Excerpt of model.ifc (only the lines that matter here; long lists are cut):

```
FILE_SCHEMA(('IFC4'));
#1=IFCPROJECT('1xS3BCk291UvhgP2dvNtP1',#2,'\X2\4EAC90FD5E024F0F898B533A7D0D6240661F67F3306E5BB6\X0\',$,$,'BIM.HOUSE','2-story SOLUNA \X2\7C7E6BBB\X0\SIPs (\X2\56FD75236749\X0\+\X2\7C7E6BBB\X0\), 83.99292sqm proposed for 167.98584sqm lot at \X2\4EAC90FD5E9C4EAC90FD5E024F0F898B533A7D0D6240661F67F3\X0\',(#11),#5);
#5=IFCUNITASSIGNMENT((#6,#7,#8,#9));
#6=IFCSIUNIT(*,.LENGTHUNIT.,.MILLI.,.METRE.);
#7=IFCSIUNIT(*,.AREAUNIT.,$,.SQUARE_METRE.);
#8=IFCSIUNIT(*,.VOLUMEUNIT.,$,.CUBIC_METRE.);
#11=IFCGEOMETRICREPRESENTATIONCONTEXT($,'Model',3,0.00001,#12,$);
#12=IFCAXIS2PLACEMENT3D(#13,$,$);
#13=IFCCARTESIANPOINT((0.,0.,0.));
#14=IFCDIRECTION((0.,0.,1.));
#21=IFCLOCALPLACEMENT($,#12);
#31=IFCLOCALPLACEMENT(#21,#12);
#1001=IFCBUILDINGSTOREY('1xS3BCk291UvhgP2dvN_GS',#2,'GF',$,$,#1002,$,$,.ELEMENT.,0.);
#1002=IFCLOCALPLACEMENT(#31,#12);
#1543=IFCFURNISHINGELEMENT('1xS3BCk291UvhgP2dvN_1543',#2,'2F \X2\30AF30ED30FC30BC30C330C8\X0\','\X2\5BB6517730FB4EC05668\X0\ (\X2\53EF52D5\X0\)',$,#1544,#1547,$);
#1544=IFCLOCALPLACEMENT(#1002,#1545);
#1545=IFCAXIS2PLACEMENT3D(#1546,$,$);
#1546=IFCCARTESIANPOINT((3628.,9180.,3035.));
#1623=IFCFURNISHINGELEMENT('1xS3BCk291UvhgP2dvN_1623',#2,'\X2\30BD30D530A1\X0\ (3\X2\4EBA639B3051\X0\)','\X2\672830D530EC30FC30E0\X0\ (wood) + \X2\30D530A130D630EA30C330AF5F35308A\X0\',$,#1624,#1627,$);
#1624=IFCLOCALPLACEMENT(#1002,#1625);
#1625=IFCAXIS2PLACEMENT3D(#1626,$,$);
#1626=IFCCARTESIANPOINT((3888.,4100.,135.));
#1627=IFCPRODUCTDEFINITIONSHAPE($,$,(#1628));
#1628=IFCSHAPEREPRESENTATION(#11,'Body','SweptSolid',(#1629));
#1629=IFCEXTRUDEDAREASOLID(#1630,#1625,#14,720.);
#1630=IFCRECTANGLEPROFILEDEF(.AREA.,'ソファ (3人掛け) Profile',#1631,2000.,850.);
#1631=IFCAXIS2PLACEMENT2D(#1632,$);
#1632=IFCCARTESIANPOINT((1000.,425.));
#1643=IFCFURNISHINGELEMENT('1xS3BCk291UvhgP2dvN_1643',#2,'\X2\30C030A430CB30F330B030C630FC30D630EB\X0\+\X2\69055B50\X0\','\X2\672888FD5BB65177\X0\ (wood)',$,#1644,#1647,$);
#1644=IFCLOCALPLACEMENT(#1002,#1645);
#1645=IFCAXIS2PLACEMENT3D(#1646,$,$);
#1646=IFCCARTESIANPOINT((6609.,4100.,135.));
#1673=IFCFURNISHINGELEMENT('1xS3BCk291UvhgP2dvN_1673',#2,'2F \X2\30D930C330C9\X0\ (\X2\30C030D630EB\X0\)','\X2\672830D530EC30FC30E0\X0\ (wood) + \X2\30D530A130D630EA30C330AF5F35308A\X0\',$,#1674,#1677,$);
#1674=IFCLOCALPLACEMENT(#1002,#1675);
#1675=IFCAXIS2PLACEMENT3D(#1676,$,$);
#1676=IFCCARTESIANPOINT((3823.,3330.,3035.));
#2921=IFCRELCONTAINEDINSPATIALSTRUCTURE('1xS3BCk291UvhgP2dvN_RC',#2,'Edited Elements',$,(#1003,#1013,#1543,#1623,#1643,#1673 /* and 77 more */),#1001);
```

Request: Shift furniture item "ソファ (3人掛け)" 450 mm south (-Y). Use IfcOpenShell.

```python
import ifcopenshell
import ifcopenshell.api.geometry
import ifcopenshell.util.placement

model = ifcopenshell.open("model.ifc")

item = model.by_id(1623)
matrix = ifcopenshell.util.placement.get_local_placement(item.ObjectPlacement)
matrix[1, 3] -= 450.0
ifcopenshell.api.geometry.edit_object_placement(model, product=item, matrix=matrix, is_si=False)

print(ifcopenshell.util.placement.get_local_placement(item.ObjectPlacement).round(3) + 0.0)

model.write("model_updated.ifc")
```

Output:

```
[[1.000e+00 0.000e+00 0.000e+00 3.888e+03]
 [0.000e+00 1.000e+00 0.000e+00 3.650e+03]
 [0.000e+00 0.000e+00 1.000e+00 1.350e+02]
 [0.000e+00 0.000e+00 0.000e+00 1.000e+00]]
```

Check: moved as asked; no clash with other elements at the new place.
